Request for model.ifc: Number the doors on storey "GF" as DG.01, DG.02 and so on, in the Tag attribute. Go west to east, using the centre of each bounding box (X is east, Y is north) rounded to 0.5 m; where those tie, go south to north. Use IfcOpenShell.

First a look at what the model holds.

```python
import ifcopenshell
import ifcopenshell.util.element
import ifcopenshell.util.placement

model = ifcopenshell.open("model.ifc")
print(model.schema)
storey = next(s for s in model.by_type("IfcBuildingStorey") if s.Name == "GF")
doors = [e for e in ifcopenshell.util.element.get_decomposition(storey) if e.is_a("IfcDoor")]
for e in sorted(doors, key=lambda e: e.id()):
    origin = ifcopenshell.util.placement.get_local_placement(e.ObjectPlacement)[:3, 3]
    print(e.id(), e.Tag, e.Name, origin.round(2) + 0.0, sep=" | ")
```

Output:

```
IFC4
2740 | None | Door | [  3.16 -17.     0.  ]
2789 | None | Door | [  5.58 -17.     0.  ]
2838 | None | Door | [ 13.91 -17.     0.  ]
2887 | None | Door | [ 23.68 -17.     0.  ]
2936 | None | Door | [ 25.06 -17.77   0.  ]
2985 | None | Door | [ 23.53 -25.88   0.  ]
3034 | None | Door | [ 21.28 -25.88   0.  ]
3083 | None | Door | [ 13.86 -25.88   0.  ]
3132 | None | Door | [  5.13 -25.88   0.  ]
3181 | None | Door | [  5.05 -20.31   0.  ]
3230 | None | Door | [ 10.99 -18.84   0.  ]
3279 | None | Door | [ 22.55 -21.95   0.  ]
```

```python
import ifcopenshell
import ifcopenshell.geom
import ifcopenshell.util.element
import ifcopenshell.util.shape

model = ifcopenshell.open("model.ifc")
settings = ifcopenshell.geom.settings()
settings.set("use-world-coords", True)


def centre(element):
    shape = ifcopenshell.geom.create_shape(settings, element)
    return ifcopenshell.util.shape.get_bbox_centroid(shape.geometry)


storey = next(s for s in model.by_type("IfcBuildingStorey") if s.Name == "GF")
doors = [e for e in ifcopenshell.util.element.get_decomposition(storey) if e.is_a("IfcDoor")]

# Insertion points can sit at a corner or the storey origin, so sort by the geometry (in metres).
centres = {e: centre(e) for e in doors}
doors.sort(key=lambda e: (round(centres[e][0] / 0.5), centres[e][1]))

for i, e in enumerate(doors, start=1):
    number = f"DG.{i:02d}"
    e.Tag = number
    print(e.id(), number)

model.write("model-out.ifc")
```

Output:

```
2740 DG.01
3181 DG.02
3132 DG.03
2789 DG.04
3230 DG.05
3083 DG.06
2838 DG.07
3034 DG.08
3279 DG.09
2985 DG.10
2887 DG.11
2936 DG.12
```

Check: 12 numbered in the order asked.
